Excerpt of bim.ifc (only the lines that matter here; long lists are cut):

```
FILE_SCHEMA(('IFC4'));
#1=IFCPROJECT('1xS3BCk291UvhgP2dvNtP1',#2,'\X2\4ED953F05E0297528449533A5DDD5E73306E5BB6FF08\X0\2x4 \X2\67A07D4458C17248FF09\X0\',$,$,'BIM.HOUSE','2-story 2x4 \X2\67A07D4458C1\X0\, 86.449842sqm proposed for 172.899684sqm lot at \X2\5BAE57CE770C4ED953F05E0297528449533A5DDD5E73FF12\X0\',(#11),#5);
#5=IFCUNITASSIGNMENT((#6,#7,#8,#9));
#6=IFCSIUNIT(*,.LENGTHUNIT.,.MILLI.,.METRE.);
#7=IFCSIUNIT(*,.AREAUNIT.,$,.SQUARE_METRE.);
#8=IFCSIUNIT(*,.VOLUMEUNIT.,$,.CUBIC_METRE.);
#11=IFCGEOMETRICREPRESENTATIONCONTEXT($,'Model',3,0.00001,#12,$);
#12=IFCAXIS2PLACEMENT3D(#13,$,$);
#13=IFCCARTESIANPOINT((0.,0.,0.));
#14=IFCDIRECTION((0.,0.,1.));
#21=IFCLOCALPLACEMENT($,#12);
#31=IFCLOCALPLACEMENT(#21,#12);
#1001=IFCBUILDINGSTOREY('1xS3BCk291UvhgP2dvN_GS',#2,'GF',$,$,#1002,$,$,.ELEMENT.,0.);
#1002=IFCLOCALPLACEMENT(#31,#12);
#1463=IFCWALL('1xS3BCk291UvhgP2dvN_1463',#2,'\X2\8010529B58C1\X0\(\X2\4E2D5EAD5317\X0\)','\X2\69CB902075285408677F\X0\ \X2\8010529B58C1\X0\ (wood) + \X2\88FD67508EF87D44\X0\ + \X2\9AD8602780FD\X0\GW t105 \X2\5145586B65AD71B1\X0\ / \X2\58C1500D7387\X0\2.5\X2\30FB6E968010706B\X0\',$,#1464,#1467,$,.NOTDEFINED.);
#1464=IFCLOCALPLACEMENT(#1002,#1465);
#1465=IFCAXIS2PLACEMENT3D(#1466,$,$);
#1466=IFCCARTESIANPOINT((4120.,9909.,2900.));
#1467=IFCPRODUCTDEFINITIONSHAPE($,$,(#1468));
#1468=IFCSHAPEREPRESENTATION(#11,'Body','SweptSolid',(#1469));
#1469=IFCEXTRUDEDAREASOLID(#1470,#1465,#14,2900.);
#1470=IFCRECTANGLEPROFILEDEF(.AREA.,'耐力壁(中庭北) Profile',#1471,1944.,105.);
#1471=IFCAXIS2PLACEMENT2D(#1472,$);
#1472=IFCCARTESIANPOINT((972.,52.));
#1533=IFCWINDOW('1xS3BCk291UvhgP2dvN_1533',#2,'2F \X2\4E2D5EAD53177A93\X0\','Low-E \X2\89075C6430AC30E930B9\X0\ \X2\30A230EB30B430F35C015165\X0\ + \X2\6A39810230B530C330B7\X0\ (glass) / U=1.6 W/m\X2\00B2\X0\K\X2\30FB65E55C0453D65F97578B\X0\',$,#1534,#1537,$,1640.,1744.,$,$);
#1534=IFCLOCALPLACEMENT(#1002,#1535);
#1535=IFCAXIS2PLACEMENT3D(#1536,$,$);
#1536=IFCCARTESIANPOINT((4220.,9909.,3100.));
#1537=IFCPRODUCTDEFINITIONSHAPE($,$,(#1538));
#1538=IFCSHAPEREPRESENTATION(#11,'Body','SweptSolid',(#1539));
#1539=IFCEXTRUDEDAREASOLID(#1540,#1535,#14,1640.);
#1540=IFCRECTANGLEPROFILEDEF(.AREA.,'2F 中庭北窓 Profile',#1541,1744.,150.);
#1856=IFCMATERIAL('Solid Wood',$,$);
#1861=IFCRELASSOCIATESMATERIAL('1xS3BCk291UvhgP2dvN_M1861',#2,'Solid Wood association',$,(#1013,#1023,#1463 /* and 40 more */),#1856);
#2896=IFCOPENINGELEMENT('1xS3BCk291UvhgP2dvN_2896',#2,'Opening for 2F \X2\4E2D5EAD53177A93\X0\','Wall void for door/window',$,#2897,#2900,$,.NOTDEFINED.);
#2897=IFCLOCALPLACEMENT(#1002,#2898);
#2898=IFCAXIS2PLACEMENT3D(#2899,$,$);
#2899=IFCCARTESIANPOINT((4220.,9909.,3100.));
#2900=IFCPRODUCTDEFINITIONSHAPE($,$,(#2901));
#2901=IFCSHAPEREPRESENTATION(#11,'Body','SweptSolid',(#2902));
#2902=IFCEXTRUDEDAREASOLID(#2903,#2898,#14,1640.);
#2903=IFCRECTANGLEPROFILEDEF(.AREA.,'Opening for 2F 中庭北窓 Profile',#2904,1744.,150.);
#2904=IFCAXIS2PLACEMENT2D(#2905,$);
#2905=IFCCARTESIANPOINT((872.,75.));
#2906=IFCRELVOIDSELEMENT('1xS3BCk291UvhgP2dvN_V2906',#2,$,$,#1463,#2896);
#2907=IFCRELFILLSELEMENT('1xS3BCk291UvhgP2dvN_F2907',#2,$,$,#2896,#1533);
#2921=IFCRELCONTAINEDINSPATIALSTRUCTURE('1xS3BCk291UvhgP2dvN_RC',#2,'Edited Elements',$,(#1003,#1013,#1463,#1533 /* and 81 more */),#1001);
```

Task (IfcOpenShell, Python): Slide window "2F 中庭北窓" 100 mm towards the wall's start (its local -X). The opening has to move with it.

```python
import ifcopenshell
import ifcopenshell.api.geometry
import ifcopenshell.util.placement
import ifcopenshell.util.unit

model = ifcopenshell.open("bim.ifc")
unit_scale = ifcopenshell.util.unit.calculate_unit_scale(model)

window = model.by_guid("1xS3BCk291UvhgP2dvN_1533")
opening = window.FillsVoids[0].RelatingOpeningElement
wall = opening.VoidsElements[0].RelatingBuildingElement

wall_matrix = ifcopenshell.util.placement.get_local_placement(wall.ObjectPlacement)
shift = wall_matrix[:3, 0] * -0.1 / unit_scale
before = ifcopenshell.util.placement.get_local_placement(window.ObjectPlacement)[:3, 3].copy()

# The window is not placed relative to its opening, so move both.
for product in (opening, window):
    matrix = ifcopenshell.util.placement.get_local_placement(product.ObjectPlacement)
    matrix[:3, 3] += shift
    ifcopenshell.api.geometry.edit_object_placement(model, product=product, matrix=matrix, is_si=False)

after = ifcopenshell.util.placement.get_local_placement(window.ObjectPlacement)[:3, 3]
print("window moved by", (after - before).round(3) + 0.0)

model.write("bim-out.ifc")
```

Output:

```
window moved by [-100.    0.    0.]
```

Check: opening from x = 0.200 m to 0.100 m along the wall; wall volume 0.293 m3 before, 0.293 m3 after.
